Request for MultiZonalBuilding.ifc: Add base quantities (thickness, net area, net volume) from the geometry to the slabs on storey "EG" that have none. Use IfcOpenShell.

First a look at what the model holds.

```python
import ifcopenshell
import ifcopenshell.util.element
import ifcopenshell.util.unit

model = ifcopenshell.open("MultiZonalBuilding.ifc")
print(model.schema)
for unit_type in ("LENGTHUNIT", "AREAUNIT", "VOLUMEUNIT"):
    print(unit_type, ifcopenshell.util.unit.calculate_unit_scale(model, unit_type))
storey = next(s for s in model.by_type("IfcBuildingStorey") if s.Name == "EG")
slabs = [e for e in ifcopenshell.util.element.get_decomposition(storey) if e.is_a("IfcSlab")]
for e in sorted(slabs, key=lambda e: e.id()):
    print(e.id(), e.is_a(), e.Name, list(ifcopenshell.util.element.get_psets(e, qtos_only=True)), sep=" | ")
```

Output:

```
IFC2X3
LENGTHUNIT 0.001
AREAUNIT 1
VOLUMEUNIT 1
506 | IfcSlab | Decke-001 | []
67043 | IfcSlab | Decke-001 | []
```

```python
import ifcopenshell
import ifcopenshell.api.pset
import ifcopenshell.geom
import ifcopenshell.util.element
import ifcopenshell.util.shape
import ifcopenshell.util.unit

model = ifcopenshell.open("MultiZonalBuilding.ifc")
unit_scale = ifcopenshell.util.unit.calculate_unit_scale(model)
area_scale = ifcopenshell.util.unit.calculate_unit_scale(model, "AREAUNIT")
volume_scale = ifcopenshell.util.unit.calculate_unit_scale(model, "VOLUMEUNIT")
settings = ifcopenshell.geom.settings()

storey = next(s for s in model.by_type("IfcBuildingStorey") if s.Name == "EG")
slabs = [e for e in ifcopenshell.util.element.get_decomposition(storey) if e.is_a("IfcSlab")]

for e in sorted(slabs, key=lambda e: e.id()):
    if ifcopenshell.util.element.get_psets(e, qtos_only=True, should_inherit=False):
        continue
    # Geometry comes back in metres, in the element's own axes.
    shape = ifcopenshell.geom.create_shape(settings, e)
    values = {
        "Width": ifcopenshell.util.shape.get_z(shape.geometry) / unit_scale,
        "NetArea": ifcopenshell.util.shape.get_footprint_area(shape.geometry) / area_scale,
        "NetVolume": ifcopenshell.util.shape.get_volume(shape.geometry) / volume_scale,
    }
    qto = ifcopenshell.api.pset.add_qto(model, product=e, name="BaseQuantities")
    ifcopenshell.api.pset.edit_qto(model, qto=qto, properties=values)
    print(e.id(), {k: round(v, 3) for k, v in values.items()})

model.write("MultiZonalBuilding-out.ifc")
```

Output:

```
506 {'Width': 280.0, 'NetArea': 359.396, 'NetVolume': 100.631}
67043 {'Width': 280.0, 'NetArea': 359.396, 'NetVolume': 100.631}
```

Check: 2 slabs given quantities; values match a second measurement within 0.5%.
